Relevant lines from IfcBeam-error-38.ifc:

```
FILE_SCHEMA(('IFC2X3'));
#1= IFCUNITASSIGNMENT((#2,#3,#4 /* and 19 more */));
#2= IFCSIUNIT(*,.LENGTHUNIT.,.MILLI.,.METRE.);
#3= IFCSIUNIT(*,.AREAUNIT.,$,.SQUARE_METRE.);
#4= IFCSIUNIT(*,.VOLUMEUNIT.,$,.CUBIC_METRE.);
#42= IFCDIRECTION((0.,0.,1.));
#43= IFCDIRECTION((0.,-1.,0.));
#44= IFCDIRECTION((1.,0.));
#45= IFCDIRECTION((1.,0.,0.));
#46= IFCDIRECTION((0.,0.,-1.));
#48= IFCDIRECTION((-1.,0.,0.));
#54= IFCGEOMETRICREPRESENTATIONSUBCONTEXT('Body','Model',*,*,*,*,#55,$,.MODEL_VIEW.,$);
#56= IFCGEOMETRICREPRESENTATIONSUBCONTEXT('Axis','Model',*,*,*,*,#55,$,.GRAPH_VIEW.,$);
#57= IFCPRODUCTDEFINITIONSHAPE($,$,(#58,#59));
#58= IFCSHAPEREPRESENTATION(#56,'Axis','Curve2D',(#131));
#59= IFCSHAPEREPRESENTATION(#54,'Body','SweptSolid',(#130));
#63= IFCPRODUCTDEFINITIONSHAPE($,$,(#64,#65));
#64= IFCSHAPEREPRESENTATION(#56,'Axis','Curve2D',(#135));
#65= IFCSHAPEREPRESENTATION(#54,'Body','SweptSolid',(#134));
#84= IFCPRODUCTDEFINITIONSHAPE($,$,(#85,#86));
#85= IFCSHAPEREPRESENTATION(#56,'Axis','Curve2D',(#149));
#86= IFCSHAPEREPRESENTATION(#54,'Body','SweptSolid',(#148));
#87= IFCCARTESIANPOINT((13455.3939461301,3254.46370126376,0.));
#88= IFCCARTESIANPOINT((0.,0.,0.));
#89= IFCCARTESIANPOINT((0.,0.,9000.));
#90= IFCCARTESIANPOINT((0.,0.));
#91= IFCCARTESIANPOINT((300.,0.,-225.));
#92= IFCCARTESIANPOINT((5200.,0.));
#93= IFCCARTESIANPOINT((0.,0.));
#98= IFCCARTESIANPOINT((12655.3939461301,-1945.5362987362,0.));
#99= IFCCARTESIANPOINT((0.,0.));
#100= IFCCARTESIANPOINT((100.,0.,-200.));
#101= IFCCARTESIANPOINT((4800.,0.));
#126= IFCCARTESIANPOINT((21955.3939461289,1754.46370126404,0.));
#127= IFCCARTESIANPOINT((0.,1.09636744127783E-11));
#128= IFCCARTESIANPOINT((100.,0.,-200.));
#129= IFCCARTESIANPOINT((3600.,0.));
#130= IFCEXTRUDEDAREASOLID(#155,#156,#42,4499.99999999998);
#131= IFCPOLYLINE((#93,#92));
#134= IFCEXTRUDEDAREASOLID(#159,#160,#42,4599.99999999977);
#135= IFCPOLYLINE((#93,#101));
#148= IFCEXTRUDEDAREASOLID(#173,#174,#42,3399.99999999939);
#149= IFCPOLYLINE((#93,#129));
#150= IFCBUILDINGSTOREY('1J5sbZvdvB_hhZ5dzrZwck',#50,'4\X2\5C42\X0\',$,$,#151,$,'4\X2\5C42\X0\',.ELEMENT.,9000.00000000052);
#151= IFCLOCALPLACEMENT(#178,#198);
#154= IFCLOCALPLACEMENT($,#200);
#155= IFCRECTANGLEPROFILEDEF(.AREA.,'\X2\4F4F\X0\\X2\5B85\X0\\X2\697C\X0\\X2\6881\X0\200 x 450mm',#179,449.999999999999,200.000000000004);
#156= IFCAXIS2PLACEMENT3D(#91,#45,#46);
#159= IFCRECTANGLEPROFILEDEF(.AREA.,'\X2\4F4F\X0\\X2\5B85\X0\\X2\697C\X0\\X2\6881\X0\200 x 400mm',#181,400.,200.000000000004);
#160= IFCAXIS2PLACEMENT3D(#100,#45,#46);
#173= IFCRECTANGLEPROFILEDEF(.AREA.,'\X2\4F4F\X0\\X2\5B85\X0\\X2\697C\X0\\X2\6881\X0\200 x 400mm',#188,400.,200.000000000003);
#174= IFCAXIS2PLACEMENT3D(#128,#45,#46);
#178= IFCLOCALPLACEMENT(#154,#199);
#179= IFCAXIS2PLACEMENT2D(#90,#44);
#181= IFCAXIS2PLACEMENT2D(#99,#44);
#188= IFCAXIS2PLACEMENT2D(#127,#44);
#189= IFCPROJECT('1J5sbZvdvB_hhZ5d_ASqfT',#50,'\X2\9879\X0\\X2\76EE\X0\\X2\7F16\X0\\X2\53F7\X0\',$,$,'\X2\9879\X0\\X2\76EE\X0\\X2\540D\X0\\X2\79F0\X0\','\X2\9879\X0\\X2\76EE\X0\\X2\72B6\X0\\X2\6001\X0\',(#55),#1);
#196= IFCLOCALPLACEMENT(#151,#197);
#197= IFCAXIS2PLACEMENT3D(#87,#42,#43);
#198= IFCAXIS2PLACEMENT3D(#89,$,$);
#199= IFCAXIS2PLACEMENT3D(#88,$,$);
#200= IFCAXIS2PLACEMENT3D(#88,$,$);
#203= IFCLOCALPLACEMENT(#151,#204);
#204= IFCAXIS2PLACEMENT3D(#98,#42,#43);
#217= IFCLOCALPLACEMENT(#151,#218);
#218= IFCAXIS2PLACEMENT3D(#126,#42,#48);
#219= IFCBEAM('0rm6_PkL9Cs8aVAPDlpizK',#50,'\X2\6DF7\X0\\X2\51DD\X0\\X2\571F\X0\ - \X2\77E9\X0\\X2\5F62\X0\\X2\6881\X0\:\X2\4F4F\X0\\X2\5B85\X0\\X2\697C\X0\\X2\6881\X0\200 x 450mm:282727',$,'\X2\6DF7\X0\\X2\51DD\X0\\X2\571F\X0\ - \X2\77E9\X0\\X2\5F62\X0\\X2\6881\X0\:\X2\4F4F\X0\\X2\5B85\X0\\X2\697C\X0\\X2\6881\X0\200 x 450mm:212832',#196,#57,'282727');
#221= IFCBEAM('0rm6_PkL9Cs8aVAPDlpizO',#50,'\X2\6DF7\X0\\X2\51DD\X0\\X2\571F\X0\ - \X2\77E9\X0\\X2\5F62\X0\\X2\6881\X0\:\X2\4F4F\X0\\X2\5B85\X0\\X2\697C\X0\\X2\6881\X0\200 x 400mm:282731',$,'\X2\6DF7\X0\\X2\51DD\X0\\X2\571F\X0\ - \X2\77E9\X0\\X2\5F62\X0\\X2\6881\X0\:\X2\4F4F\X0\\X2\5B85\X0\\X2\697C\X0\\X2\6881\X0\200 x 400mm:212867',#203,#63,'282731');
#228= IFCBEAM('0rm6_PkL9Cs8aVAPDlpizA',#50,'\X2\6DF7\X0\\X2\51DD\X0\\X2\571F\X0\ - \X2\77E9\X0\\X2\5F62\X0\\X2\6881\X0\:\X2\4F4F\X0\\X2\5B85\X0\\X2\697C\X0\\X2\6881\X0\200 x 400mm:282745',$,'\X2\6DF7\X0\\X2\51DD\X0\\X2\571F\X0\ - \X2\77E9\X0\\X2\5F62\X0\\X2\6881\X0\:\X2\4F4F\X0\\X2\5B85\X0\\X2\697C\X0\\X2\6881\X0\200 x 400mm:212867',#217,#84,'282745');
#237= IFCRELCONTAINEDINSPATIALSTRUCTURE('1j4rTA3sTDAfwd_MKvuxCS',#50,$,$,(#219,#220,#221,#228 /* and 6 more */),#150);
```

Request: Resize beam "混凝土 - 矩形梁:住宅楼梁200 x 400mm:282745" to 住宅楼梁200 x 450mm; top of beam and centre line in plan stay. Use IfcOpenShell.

```python
import ifcopenshell
import ifcopenshell.util.element
import ifcopenshell.util.representation

model = ifcopenshell.open("IfcBeam-error-38.ifc")

member = model.by_guid("0rm6_PkL9Cs8aVAPDlpizA")
source = next(p for p in model.by_type("IfcRectangleProfileDef") if p.ProfileName == "住宅楼梁200 x 450mm")

body = ifcopenshell.util.representation.get_representation(member, "Model", "Body")
solid = body.Items[0]
old_profile = solid.SweptArea

# Copy the section's sizes but keep this member's own profile position.
profile = ifcopenshell.util.element.copy(model, source)
# Profiles are centred, so shift by half the change in depth to hold the top.
shift = (old_profile.XDim - profile.XDim) / 2
x, y = old_profile.Position.Location.Coordinates
up = (-1.0, 0.0)  # upwards, in the solid's own plane
location = model.createIfcCartesianPoint((x + up[0] * shift, y + up[1] * shift))
profile.Position = model.createIfcAxis2Placement2D(location, old_profile.Position.RefDirection)
solid.SweptArea = profile
if not model.get_total_inverses(old_profile):
    ifcopenshell.util.element.remove_deep2(model, old_profile)
member.Name = member.Name.replace("住宅楼梁200 x 400mm", "住宅楼梁200 x 450mm")
member.ObjectType = member.ObjectType.replace("住宅楼梁200 x 400mm", "住宅楼梁200 x 450mm")

print(solid.SweptArea)

model.write("IfcBeam-error-38_updated.ifc")
```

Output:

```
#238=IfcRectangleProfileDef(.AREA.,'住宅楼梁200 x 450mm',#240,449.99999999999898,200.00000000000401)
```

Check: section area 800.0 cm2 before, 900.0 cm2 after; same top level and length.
